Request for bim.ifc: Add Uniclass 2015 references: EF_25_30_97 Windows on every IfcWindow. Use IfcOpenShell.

First a look at what the model holds.

```python
import ifcopenshell

model = ifcopenshell.open("bim.ifc")
print(model.schema)
print("classifications:", [c.Name for c in model.by_type("IfcClassification")])
for ifc_class in ("IfcDoor", "IfcRoof", "IfcStair", "IfcWall", "IfcWindow"):
    print(ifc_class, len(model.by_type(ifc_class)))
```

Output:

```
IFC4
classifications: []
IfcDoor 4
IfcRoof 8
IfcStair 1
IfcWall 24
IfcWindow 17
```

```python
import ifcopenshell
import ifcopenshell.api.classification

model = ifcopenshell.open("bim.ifc")

system = ifcopenshell.api.classification.add_classification(model, classification="Uniclass 2015")

codes = {
    "IfcWindow": ("EF_25_30_97", "Windows"),
}
for ifc_class, (code, name) in codes.items():
    products = model.by_type(ifc_class)
    ifcopenshell.api.classification.add_reference(
        model, products=products, classification=system, identification=code, name=name
    )
    print(code, len(products))

model.write("bim_v2.ifc")
```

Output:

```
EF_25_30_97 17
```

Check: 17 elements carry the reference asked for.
